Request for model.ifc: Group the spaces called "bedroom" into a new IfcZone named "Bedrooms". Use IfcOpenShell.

First a look at what the model holds.

```python
import ifcopenshell

model = ifcopenshell.open("model.ifc")
print(model.schema)
seen = {}
for space in model.by_type("IfcSpace"):
    seen[space.LongName] = seen.get(space.LongName, 0) + 1
for name, count in sorted(seen.items(), key=str):
    print(count, "x", name)
print("zones:", [z.Name for z in model.by_type("IfcZone")][:20])
```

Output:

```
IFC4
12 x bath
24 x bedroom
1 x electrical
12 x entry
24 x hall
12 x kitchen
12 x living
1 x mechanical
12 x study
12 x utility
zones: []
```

```python
import ifcopenshell
import ifcopenshell.api.group
import ifcopenshell.api.root

model = ifcopenshell.open("model.ifc")

names = {"bedroom"}
spaces = [s for s in model.by_type("IfcSpace") if s.LongName in names]

zone = ifcopenshell.api.root.create_entity(model, ifc_class="IfcZone", name="Bedrooms")
ifcopenshell.api.group.assign_group(model, products=spaces, group=zone)
print(len(spaces), "spaces in", zone.Name)

model.write("model_edited.ifc")
```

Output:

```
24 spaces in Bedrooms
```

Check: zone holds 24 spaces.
